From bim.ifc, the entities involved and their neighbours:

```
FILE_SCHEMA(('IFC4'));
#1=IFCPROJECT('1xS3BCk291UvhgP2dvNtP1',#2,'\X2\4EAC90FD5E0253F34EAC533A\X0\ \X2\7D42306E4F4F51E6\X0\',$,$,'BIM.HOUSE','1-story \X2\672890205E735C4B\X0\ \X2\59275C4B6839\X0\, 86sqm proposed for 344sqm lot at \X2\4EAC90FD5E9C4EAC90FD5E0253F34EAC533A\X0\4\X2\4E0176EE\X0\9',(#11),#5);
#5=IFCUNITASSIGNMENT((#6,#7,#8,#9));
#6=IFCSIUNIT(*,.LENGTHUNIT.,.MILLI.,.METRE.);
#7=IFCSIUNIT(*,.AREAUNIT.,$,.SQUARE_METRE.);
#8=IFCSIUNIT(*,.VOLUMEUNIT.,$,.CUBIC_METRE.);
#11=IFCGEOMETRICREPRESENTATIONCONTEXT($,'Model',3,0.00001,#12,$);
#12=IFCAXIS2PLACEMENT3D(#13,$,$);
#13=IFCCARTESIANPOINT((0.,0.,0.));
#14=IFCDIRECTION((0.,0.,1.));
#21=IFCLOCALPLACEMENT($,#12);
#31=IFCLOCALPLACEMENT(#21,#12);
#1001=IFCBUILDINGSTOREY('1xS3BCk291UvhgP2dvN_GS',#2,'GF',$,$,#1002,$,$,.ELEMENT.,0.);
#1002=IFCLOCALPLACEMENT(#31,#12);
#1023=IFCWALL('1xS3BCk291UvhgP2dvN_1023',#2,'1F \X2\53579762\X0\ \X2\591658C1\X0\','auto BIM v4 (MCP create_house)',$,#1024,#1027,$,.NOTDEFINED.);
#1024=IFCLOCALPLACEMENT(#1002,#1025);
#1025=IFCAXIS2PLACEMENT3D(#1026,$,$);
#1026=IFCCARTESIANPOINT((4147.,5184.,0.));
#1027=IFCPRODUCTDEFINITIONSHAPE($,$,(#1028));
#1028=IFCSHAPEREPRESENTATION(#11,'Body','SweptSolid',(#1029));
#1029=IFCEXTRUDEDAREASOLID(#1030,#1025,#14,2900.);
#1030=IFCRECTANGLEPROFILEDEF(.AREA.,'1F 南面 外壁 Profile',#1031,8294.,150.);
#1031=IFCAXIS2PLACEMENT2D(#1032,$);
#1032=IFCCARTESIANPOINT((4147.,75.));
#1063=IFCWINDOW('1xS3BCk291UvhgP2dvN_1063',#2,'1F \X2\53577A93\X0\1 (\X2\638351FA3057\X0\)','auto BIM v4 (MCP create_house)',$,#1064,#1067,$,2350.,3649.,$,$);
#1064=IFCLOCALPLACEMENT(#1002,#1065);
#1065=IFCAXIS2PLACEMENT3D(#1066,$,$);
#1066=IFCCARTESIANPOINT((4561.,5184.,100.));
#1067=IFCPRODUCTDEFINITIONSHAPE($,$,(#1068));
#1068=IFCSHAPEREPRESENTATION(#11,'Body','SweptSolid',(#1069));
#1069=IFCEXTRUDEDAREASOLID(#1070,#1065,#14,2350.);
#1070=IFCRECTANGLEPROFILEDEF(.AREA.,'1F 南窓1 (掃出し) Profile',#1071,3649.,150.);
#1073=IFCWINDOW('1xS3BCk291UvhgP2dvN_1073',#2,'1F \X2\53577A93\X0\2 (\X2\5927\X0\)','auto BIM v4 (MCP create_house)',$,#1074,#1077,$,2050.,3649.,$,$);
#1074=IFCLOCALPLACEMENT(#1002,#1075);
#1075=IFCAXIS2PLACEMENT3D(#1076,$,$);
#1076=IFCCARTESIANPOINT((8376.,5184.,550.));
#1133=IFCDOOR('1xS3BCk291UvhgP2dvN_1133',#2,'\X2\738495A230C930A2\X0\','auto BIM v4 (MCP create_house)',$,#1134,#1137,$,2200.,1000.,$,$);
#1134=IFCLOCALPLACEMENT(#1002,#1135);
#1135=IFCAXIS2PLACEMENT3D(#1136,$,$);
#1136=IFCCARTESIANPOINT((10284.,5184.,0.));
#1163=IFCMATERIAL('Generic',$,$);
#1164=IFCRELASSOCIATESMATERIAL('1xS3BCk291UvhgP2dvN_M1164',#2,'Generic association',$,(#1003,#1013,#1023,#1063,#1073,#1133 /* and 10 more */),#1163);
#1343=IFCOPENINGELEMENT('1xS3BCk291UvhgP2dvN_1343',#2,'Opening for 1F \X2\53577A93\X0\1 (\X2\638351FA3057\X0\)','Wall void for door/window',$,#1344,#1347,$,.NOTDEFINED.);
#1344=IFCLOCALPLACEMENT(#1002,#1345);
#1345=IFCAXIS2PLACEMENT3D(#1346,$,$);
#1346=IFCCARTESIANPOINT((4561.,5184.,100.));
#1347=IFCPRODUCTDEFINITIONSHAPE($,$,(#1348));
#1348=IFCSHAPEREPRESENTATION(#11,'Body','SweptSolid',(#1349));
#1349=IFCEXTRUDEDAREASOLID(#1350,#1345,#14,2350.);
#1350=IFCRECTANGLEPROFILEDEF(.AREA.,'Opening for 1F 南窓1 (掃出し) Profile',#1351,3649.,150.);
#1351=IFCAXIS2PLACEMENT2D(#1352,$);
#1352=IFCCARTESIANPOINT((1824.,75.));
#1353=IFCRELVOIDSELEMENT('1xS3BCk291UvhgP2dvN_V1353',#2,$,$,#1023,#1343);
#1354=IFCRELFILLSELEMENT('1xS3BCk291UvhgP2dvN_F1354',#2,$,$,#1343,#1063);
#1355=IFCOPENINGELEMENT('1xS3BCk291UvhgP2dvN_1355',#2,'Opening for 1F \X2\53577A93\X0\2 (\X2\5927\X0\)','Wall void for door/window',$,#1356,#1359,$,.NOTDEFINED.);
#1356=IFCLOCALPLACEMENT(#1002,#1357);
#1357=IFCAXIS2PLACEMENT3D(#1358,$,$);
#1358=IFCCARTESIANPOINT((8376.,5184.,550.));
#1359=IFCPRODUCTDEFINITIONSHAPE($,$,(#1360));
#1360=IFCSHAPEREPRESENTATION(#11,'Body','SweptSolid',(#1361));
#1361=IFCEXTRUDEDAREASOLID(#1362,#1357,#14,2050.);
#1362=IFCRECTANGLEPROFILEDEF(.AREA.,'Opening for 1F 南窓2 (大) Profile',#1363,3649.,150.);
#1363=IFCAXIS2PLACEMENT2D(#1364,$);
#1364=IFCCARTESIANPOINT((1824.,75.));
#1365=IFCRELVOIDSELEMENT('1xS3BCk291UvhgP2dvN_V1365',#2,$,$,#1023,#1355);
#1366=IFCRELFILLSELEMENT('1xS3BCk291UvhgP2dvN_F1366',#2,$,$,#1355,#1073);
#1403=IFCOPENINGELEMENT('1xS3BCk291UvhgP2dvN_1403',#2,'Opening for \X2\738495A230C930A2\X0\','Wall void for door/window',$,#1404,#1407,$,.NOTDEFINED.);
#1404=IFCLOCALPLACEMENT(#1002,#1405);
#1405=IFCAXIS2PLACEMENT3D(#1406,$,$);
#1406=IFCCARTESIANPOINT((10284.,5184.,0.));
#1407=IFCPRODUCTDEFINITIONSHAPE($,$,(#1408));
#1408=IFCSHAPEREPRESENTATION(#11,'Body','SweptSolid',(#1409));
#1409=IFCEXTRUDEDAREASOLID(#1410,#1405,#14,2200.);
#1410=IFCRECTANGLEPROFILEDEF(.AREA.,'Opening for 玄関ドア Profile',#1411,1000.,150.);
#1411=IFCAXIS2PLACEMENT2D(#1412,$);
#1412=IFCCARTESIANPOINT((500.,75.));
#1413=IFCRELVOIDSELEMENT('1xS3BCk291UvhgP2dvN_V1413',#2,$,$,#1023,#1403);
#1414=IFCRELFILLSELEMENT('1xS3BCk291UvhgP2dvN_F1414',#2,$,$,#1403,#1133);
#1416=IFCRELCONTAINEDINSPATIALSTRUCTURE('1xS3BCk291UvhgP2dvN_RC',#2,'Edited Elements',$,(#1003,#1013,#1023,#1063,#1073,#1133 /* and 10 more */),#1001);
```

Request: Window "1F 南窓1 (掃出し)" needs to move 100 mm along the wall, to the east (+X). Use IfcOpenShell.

```python
import ifcopenshell
import ifcopenshell.api.geometry
import ifcopenshell.util.placement
import ifcopenshell.util.unit

model = ifcopenshell.open("bim.ifc")
unit_scale = ifcopenshell.util.unit.calculate_unit_scale(model)

window = model.by_guid("1xS3BCk291UvhgP2dvN_1063")
opening = window.FillsVoids[0].RelatingOpeningElement
wall = opening.VoidsElements[0].RelatingBuildingElement

wall_matrix = ifcopenshell.util.placement.get_local_placement(wall.ObjectPlacement)
shift = wall_matrix[:3, 0] * 0.1 / unit_scale
before = ifcopenshell.util.placement.get_local_placement(window.ObjectPlacement)[:3, 3].copy()

# The window is not placed relative to its opening, so move both.
for product in (opening, window):
    matrix = ifcopenshell.util.placement.get_local_placement(product.ObjectPlacement)
    matrix[:3, 3] += shift
    ifcopenshell.api.geometry.edit_object_placement(model, product=product, matrix=matrix, is_si=False)

after = ifcopenshell.util.placement.get_local_placement(window.ObjectPlacement)[:3, 3]
print("window moved by", (after - before).round(3) + 0.0)

model.write("bim_v2.ifc")
```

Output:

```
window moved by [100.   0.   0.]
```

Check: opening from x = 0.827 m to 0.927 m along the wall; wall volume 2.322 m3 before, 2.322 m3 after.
